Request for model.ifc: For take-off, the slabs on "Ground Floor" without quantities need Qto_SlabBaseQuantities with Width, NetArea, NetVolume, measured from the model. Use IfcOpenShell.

First a look at what the model holds.

```python
import ifcopenshell
import ifcopenshell.util.element
import ifcopenshell.util.unit

model = ifcopenshell.open("model.ifc")
print(model.schema)
for unit_type in ("LENGTHUNIT", "AREAUNIT", "VOLUMEUNIT"):
    print(unit_type, ifcopenshell.util.unit.calculate_unit_scale(model, unit_type))
storey = next(s for s in model.by_type("IfcBuildingStorey") if s.Name == "Ground Floor")
slabs = [e for e in ifcopenshell.util.element.get_decomposition(storey) if e.is_a("IfcSlab")]
for e in sorted(slabs, key=lambda e: e.id()):
    print(e.id(), e.is_a(), e.Name, list(ifcopenshell.util.element.get_psets(e, qtos_only=True)), sep=" | ")
```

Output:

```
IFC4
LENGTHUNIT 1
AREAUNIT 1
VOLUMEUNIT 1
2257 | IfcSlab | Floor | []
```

```python
import ifcopenshell
import ifcopenshell.api.pset
import ifcopenshell.geom
import ifcopenshell.util.element
import ifcopenshell.util.shape
import ifcopenshell.util.unit

model = ifcopenshell.open("model.ifc")
unit_scale = ifcopenshell.util.unit.calculate_unit_scale(model)
area_scale = ifcopenshell.util.unit.calculate_unit_scale(model, "AREAUNIT")
volume_scale = ifcopenshell.util.unit.calculate_unit_scale(model, "VOLUMEUNIT")
settings = ifcopenshell.geom.settings()

storey = next(s for s in model.by_type("IfcBuildingStorey") if s.Name == "Ground Floor")
slabs = [e for e in ifcopenshell.util.element.get_decomposition(storey) if e.is_a("IfcSlab")]

for e in sorted(slabs, key=lambda e: e.id()):
    if ifcopenshell.util.element.get_psets(e, qtos_only=True, should_inherit=False):
        continue
    # Geometry comes back in metres, in the element's own axes.
    shape = ifcopenshell.geom.create_shape(settings, e)
    values = {
        "Width": ifcopenshell.util.shape.get_z(shape.geometry) / unit_scale,
        "NetArea": ifcopenshell.util.shape.get_footprint_area(shape.geometry) / area_scale,
        "NetVolume": ifcopenshell.util.shape.get_volume(shape.geometry) / volume_scale,
    }
    qto = ifcopenshell.api.pset.add_qto(model, product=e, name="Qto_SlabBaseQuantities")
    ifcopenshell.api.pset.edit_qto(model, qto=qto, properties=values)
    print(e.id(), {k: round(v, 3) for k, v in values.items()})

model.write("model_rev.ifc")
```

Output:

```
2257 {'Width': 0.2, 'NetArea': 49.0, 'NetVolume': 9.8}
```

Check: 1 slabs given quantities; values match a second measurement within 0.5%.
